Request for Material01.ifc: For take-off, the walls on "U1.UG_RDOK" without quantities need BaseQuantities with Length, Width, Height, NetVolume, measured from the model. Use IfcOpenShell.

First a look at what the model holds.

```python
import ifcopenshell
import ifcopenshell.util.element
import ifcopenshell.util.unit

model = ifcopenshell.open("Material01.ifc")
print(model.schema)
for unit_type in ("LENGTHUNIT", "AREAUNIT", "VOLUMEUNIT"):
    print(unit_type, ifcopenshell.util.unit.calculate_unit_scale(model, unit_type))
storey = next(s for s in model.by_type("IfcBuildingStorey") if s.Name == "U1.UG_RDOK")
walls = [e for e in ifcopenshell.util.element.get_decomposition(storey) if e.is_a("IfcWall")]
for e in sorted(walls, key=lambda e: e.id()):
    print(e.id(), e.is_a(), e.Name, list(ifcopenshell.util.element.get_psets(e, qtos_only=True)), sep=" | ")
```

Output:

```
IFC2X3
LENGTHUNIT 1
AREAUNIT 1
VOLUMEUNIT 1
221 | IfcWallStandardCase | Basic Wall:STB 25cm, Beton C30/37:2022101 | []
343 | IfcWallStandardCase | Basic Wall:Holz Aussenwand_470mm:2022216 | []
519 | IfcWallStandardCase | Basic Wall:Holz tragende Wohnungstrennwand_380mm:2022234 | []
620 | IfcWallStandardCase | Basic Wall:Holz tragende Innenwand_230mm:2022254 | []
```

```python
import ifcopenshell
import ifcopenshell.api.pset
import ifcopenshell.geom
import ifcopenshell.util.element
import ifcopenshell.util.shape
import ifcopenshell.util.unit

model = ifcopenshell.open("Material01.ifc")
unit_scale = ifcopenshell.util.unit.calculate_unit_scale(model)
volume_scale = ifcopenshell.util.unit.calculate_unit_scale(model, "VOLUMEUNIT")
settings = ifcopenshell.geom.settings()

storey = next(s for s in model.by_type("IfcBuildingStorey") if s.Name == "U1.UG_RDOK")
walls = [e for e in ifcopenshell.util.element.get_decomposition(storey) if e.is_a("IfcWall")]

for e in sorted(walls, key=lambda e: e.id()):
    if ifcopenshell.util.element.get_psets(e, qtos_only=True, should_inherit=False):
        continue
    # Geometry comes back in metres, in the element's own axes.
    shape = ifcopenshell.geom.create_shape(settings, e)
    values = {
        "Length": ifcopenshell.util.shape.get_x(shape.geometry) / unit_scale,
        "Width": ifcopenshell.util.shape.get_y(shape.geometry) / unit_scale,
        "Height": ifcopenshell.util.shape.get_z(shape.geometry) / unit_scale,
        "NetVolume": ifcopenshell.util.shape.get_volume(shape.geometry) / volume_scale,
    }
    qto = ifcopenshell.api.pset.add_qto(model, product=e, name="BaseQuantities")
    ifcopenshell.api.pset.edit_qto(model, qto=qto, properties=values)
    print(e.id(), {k: round(v, 3) for k, v in values.items()})

model.write("Material01-out.ifc")
```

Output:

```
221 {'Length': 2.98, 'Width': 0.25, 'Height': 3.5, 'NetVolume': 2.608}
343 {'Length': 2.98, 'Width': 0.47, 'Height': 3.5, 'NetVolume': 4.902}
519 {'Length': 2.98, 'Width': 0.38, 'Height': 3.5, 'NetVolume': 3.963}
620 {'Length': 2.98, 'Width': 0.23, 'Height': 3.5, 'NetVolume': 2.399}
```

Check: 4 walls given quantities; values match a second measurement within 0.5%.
